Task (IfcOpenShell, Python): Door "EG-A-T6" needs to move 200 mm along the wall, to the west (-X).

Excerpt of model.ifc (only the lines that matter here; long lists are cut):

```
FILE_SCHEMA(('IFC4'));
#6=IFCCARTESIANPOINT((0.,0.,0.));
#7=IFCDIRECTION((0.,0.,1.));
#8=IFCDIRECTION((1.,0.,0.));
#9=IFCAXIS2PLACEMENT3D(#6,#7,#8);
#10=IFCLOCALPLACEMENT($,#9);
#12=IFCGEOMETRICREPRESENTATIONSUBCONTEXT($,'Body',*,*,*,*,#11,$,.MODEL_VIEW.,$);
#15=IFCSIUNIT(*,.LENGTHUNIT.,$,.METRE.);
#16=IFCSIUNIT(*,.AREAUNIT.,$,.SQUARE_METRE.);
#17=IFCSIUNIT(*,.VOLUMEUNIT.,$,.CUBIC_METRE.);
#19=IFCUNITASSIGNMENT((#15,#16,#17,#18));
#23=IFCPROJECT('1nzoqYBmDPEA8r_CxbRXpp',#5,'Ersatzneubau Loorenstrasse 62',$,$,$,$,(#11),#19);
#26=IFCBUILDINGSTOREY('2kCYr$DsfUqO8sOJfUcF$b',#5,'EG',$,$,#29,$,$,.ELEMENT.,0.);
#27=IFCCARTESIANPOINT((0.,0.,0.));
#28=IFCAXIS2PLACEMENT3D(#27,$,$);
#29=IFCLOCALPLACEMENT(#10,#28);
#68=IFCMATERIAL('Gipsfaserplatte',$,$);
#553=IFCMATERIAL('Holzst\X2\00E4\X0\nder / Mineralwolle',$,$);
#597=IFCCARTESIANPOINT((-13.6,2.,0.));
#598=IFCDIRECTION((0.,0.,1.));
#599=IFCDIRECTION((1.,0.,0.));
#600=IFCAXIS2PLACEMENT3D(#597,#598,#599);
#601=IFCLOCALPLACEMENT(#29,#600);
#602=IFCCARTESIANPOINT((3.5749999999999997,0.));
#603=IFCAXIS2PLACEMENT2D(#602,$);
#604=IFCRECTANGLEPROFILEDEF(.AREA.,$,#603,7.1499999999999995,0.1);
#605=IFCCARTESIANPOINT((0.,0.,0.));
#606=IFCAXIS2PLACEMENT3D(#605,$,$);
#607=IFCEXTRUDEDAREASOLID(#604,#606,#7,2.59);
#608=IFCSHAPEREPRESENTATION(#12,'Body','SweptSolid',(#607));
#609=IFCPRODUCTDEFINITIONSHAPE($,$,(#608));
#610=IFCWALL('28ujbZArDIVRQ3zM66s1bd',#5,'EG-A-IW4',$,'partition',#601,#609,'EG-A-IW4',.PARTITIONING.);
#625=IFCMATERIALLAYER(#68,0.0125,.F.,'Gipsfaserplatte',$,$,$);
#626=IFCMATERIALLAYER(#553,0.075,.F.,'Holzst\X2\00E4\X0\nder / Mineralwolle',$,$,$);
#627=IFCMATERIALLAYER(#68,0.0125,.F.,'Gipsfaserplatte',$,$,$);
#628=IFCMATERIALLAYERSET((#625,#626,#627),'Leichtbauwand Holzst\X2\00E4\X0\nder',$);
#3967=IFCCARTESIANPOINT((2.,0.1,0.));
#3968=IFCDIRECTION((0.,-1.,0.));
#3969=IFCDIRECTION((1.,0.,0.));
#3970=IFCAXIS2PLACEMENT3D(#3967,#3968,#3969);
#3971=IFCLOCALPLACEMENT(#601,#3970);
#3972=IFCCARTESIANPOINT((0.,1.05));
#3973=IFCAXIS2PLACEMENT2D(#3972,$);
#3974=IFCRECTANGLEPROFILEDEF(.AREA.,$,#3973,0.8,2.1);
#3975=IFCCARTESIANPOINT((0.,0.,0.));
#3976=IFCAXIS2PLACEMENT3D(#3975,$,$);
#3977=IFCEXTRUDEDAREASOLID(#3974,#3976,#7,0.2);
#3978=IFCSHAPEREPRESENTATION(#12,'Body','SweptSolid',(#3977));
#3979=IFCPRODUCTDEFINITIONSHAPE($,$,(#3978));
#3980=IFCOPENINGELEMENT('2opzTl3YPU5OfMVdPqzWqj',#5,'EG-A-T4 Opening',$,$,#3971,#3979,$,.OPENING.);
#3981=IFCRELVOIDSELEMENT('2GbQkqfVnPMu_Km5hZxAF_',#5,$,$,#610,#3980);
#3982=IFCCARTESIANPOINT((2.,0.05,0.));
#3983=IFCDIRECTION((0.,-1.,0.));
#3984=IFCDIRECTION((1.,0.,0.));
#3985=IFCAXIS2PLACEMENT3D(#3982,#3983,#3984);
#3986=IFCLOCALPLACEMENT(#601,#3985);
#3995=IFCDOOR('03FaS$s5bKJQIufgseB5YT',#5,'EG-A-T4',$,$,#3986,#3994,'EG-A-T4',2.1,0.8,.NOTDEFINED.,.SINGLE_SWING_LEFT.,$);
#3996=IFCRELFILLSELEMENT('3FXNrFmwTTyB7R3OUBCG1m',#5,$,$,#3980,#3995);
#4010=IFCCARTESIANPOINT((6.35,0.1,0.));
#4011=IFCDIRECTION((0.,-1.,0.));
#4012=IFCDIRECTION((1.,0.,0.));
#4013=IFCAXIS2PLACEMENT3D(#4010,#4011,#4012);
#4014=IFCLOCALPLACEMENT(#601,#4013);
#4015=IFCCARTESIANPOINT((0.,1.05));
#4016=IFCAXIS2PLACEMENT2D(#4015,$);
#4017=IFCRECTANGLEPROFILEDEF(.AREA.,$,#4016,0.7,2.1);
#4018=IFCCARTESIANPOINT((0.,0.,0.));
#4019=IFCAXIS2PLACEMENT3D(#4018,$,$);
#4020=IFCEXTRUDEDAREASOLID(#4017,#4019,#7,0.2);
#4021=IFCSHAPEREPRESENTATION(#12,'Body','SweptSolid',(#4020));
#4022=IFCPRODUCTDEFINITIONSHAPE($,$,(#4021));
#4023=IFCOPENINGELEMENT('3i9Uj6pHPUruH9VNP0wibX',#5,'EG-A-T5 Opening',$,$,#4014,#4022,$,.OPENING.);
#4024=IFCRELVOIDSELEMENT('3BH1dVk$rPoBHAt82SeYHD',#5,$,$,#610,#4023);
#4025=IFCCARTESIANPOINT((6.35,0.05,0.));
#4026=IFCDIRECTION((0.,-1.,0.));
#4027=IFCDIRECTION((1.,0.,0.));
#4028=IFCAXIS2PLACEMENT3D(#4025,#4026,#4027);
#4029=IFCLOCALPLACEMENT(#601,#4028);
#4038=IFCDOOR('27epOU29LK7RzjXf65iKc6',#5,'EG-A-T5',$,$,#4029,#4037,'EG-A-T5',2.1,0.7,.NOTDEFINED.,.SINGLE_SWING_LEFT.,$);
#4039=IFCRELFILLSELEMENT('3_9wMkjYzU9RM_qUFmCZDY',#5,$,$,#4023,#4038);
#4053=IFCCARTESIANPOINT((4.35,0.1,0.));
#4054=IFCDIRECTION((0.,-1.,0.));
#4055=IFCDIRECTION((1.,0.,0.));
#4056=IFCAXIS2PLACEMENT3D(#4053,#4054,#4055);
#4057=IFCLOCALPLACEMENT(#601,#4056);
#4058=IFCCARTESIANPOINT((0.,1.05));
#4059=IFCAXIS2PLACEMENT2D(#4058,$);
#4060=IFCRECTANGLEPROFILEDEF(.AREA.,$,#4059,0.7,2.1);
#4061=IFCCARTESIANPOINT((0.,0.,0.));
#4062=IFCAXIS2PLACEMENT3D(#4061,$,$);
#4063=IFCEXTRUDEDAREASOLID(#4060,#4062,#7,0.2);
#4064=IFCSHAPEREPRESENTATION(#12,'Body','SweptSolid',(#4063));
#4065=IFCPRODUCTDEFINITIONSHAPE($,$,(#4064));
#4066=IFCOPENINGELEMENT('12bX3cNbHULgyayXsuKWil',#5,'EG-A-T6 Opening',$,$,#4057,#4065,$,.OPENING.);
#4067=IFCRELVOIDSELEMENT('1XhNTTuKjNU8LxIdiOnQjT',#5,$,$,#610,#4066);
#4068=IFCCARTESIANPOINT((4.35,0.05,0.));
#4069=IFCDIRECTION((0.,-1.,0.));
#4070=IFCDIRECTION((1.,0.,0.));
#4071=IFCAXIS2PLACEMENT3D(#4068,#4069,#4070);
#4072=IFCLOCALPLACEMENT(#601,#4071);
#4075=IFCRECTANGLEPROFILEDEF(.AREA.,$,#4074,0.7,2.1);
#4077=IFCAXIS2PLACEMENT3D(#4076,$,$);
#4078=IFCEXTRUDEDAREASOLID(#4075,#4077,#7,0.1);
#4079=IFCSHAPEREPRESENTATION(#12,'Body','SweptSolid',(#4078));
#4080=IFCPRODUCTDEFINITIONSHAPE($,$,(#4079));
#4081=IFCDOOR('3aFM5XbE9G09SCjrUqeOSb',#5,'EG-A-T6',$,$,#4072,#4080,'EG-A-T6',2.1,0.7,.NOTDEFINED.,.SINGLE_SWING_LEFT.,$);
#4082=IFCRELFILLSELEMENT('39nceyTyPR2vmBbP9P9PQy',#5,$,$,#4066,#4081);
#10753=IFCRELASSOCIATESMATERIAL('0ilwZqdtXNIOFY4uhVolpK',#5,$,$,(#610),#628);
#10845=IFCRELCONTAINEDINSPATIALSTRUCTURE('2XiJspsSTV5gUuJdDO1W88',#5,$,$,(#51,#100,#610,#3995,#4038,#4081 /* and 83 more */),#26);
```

```python
import ifcopenshell
import ifcopenshell.api.geometry
import ifcopenshell.util.placement
import ifcopenshell.util.unit

model = ifcopenshell.open("model.ifc")
unit_scale = ifcopenshell.util.unit.calculate_unit_scale(model)

door = model.by_guid("3aFM5XbE9G09SCjrUqeOSb")
opening = door.FillsVoids[0].RelatingOpeningElement
wall = opening.VoidsElements[0].RelatingBuildingElement

wall_matrix = ifcopenshell.util.placement.get_local_placement(wall.ObjectPlacement)
shift = wall_matrix[:3, 0] * -0.2 / unit_scale
before = ifcopenshell.util.placement.get_local_placement(door.ObjectPlacement)[:3, 3].copy()

# The door is not placed relative to its opening, so move both.
for product in (opening, door):
    matrix = ifcopenshell.util.placement.get_local_placement(product.ObjectPlacement)
    matrix[:3, 3] += shift
    ifcopenshell.api.geometry.edit_object_placement(model, product=product, matrix=matrix, is_si=False)

after = ifcopenshell.util.placement.get_local_placement(door.ObjectPlacement)[:3, 3]
print("door moved by", (after - before).round(3) + 0.0)

model.write("model_rev.ifc")
```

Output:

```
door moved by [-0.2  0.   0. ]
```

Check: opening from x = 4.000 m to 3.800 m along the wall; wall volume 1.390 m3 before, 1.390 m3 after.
